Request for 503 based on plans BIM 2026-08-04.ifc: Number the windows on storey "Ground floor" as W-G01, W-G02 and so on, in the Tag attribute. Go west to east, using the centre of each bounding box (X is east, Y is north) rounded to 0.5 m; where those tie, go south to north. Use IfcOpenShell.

First a look at what the model holds.

```python
import ifcopenshell
import ifcopenshell.util.element
import ifcopenshell.util.placement

model = ifcopenshell.open("503 based on plans BIM 2026-08-04.ifc")
print(model.schema)
storey = next(s for s in model.by_type("IfcBuildingStorey") if s.Name == "Ground floor")
windows = [e for e in ifcopenshell.util.element.get_decomposition(storey) if e.is_a("IfcWindow")]
for e in sorted(windows, key=lambda e: e.id()):
    origin = ifcopenshell.util.placement.get_local_placement(e.ObjectPlacement)[:3, 3]
    print(e.id(), e.Tag, e.Name, origin.round(2) + 0.0, sep=" | ")
```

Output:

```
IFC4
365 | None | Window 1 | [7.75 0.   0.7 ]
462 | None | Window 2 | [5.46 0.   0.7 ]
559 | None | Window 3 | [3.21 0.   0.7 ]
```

```python
import ifcopenshell
import ifcopenshell.geom
import ifcopenshell.util.element
import ifcopenshell.util.shape

model = ifcopenshell.open("503 based on plans BIM 2026-08-04.ifc")
settings = ifcopenshell.geom.settings()
settings.set("use-world-coords", True)


def centre(element):
    shape = ifcopenshell.geom.create_shape(settings, element)
    return ifcopenshell.util.shape.get_bbox_centroid(shape.geometry)


storey = next(s for s in model.by_type("IfcBuildingStorey") if s.Name == "Ground floor")
windows = [e for e in ifcopenshell.util.element.get_decomposition(storey) if e.is_a("IfcWindow")]

# Insertion points can sit at a corner or the storey origin, so sort by the geometry (in metres).
centres = {e: centre(e) for e in windows}
windows.sort(key=lambda e: (round(centres[e][0] / 0.5), centres[e][1]))

for i, e in enumerate(windows, start=1):
    number = f"W-G{i:02d}"
    e.Tag = number
    print(e.id(), number)

model.write("503 based on plans BIM 2026-08-04_updated.ifc")
```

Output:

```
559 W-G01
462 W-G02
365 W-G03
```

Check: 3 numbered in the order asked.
